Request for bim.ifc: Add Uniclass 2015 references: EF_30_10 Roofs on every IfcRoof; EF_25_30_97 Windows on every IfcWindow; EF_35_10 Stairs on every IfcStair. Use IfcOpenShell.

First a look at what the model holds.

```python
import ifcopenshell

model = ifcopenshell.open("bim.ifc")
print(model.schema)
print("classifications:", [c.Name for c in model.by_type("IfcClassification")])
for ifc_class in ("IfcDoor", "IfcRoof", "IfcStair", "IfcWall", "IfcWindow"):
    print(ifc_class, len(model.by_type(ifc_class)))
```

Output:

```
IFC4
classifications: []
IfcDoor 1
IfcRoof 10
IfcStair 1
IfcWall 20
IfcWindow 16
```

```python
import ifcopenshell
import ifcopenshell.api.classification

model = ifcopenshell.open("bim.ifc")

system = ifcopenshell.api.classification.add_classification(model, classification="Uniclass 2015")

codes = {
    "IfcRoof": ("EF_30_10", "Roofs"),
    "IfcWindow": ("EF_25_30_97", "Windows"),
    "IfcStair": ("EF_35_10", "Stairs"),
}
for ifc_class, (code, name) in codes.items():
    products = model.by_type(ifc_class)
    ifcopenshell.api.classification.add_reference(
        model, products=products, classification=system, identification=code, name=name
    )
    print(code, len(products))

model.write("bim_rev.ifc")
```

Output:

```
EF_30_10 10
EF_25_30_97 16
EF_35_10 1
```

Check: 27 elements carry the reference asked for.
